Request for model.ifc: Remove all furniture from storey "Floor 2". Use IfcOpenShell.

First a look at what the model holds.

```python
import ifcopenshell
import ifcopenshell.util.element

model = ifcopenshell.open("model.ifc")
print(model.schema)
storey = next(s for s in model.by_type("IfcBuildingStorey") if s.Name == "Floor 2")
furniture = [e for e in ifcopenshell.util.element.get_decomposition(storey) if e.is_a("IfcFurnishingElement")]
seen = {}
for e in furniture:
    element_type = ifcopenshell.util.element.get_type(e)
    name = element_type.Name if element_type not in (None, e) else None
    seen[name] = seen.get(name, 0) + 1
for name, count in sorted(seen.items(), key=str):
    print(count, "x", name)
```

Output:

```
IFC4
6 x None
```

```python
import ifcopenshell
import ifcopenshell.api.root
import ifcopenshell.util.element

model = ifcopenshell.open("model.ifc")

storey = next(s for s in model.by_type("IfcBuildingStorey") if s.Name == "Floor 2")
furniture = [e for e in ifcopenshell.util.element.get_decomposition(storey) if e.is_a("IfcFurnishingElement")]

for e in furniture:
    ifcopenshell.api.root.remove_product(model, product=e)
print(len(furniture), "removed")

model.write("model_edited.ifc")
```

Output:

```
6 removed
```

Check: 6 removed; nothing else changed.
